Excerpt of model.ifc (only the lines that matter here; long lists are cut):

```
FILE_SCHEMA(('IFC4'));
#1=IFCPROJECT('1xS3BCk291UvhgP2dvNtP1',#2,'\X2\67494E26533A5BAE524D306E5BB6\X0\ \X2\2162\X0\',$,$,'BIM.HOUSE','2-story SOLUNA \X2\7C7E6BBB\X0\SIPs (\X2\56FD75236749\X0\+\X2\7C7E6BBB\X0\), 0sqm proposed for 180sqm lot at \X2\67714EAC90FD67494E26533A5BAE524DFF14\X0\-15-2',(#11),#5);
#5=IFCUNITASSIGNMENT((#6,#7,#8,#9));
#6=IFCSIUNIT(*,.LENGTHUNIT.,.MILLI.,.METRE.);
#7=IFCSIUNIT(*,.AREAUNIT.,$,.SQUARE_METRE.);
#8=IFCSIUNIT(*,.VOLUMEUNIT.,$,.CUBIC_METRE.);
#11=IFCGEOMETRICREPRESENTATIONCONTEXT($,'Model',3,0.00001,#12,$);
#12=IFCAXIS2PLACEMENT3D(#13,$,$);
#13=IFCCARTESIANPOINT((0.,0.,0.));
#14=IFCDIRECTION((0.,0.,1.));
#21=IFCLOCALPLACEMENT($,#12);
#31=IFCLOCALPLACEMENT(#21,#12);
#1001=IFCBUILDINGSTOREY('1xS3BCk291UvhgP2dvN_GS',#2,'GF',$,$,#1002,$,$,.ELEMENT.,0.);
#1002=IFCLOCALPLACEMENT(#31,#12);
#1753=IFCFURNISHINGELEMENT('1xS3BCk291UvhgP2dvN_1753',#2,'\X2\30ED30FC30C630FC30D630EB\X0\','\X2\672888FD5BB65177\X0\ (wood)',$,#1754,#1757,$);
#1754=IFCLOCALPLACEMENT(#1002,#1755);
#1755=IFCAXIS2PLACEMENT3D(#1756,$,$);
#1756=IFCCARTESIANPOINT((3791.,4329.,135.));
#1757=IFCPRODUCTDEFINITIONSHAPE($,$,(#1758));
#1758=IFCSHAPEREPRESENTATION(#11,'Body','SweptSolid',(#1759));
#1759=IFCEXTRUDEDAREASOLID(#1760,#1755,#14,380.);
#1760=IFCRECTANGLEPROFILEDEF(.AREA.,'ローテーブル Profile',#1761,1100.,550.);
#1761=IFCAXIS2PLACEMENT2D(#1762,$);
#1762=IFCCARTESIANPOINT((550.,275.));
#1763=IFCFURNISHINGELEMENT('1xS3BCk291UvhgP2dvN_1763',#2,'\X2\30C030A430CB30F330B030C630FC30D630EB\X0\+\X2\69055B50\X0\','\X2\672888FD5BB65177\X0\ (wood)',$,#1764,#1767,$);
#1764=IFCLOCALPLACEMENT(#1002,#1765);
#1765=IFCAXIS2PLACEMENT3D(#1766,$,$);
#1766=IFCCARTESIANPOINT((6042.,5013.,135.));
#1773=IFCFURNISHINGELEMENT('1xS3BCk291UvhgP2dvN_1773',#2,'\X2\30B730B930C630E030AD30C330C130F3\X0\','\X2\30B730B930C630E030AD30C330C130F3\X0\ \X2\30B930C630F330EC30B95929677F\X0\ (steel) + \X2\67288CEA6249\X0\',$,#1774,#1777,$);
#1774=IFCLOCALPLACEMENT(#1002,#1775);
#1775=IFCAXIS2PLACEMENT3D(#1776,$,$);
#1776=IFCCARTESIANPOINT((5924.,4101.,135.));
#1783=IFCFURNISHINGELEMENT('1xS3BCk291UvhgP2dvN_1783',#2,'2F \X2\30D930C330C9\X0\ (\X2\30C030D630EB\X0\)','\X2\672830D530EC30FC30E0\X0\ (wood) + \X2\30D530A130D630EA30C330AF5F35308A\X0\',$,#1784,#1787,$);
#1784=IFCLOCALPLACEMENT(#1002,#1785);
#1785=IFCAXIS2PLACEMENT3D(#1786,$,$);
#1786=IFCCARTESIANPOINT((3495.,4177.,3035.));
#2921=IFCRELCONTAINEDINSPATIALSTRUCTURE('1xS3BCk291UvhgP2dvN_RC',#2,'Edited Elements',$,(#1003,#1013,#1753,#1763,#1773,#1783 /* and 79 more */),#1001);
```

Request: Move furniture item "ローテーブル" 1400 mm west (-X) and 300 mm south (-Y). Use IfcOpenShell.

```python
import ifcopenshell
import ifcopenshell.api.geometry
import ifcopenshell.util.placement

model = ifcopenshell.open("model.ifc")

item = model.by_id(1753)
matrix = ifcopenshell.util.placement.get_local_placement(item.ObjectPlacement)
matrix[0, 3] -= 1400.0
matrix[1, 3] -= 300.0
ifcopenshell.api.geometry.edit_object_placement(model, product=item, matrix=matrix, is_si=False)

print(ifcopenshell.util.placement.get_local_placement(item.ObjectPlacement).round(3) + 0.0)

model.write("model_edited.ifc")
```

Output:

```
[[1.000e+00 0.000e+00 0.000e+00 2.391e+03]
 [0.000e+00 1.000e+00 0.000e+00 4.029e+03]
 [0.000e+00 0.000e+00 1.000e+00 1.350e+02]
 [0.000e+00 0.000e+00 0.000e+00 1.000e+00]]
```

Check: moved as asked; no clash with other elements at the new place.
